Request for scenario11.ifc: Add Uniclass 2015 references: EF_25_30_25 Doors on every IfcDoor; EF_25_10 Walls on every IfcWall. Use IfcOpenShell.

First a look at what the model holds.

```python
import ifcopenshell

model = ifcopenshell.open("scenario11.ifc")
print(model.schema)
print("classifications:", [c.Name for c in model.by_type("IfcClassification")])
for ifc_class in ("IfcDoor", "IfcRoof", "IfcStair", "IfcWall", "IfcWindow"):
    print(ifc_class, len(model.by_type(ifc_class)))
```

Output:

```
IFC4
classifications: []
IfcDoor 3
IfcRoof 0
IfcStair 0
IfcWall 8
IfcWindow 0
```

```python
import ifcopenshell
import ifcopenshell.api.classification

model = ifcopenshell.open("scenario11.ifc")

system = ifcopenshell.api.classification.add_classification(model, classification="Uniclass 2015")

codes = {
    "IfcDoor": ("EF_25_30_25", "Doors"),
    "IfcWall": ("EF_25_10", "Walls"),
}
for ifc_class, (code, name) in codes.items():
    products = model.by_type(ifc_class)
    ifcopenshell.api.classification.add_reference(
        model, products=products, classification=system, identification=code, name=name
    )
    print(code, len(products))

model.write("scenario11_edited.ifc")
```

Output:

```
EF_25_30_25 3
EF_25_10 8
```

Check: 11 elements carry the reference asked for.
